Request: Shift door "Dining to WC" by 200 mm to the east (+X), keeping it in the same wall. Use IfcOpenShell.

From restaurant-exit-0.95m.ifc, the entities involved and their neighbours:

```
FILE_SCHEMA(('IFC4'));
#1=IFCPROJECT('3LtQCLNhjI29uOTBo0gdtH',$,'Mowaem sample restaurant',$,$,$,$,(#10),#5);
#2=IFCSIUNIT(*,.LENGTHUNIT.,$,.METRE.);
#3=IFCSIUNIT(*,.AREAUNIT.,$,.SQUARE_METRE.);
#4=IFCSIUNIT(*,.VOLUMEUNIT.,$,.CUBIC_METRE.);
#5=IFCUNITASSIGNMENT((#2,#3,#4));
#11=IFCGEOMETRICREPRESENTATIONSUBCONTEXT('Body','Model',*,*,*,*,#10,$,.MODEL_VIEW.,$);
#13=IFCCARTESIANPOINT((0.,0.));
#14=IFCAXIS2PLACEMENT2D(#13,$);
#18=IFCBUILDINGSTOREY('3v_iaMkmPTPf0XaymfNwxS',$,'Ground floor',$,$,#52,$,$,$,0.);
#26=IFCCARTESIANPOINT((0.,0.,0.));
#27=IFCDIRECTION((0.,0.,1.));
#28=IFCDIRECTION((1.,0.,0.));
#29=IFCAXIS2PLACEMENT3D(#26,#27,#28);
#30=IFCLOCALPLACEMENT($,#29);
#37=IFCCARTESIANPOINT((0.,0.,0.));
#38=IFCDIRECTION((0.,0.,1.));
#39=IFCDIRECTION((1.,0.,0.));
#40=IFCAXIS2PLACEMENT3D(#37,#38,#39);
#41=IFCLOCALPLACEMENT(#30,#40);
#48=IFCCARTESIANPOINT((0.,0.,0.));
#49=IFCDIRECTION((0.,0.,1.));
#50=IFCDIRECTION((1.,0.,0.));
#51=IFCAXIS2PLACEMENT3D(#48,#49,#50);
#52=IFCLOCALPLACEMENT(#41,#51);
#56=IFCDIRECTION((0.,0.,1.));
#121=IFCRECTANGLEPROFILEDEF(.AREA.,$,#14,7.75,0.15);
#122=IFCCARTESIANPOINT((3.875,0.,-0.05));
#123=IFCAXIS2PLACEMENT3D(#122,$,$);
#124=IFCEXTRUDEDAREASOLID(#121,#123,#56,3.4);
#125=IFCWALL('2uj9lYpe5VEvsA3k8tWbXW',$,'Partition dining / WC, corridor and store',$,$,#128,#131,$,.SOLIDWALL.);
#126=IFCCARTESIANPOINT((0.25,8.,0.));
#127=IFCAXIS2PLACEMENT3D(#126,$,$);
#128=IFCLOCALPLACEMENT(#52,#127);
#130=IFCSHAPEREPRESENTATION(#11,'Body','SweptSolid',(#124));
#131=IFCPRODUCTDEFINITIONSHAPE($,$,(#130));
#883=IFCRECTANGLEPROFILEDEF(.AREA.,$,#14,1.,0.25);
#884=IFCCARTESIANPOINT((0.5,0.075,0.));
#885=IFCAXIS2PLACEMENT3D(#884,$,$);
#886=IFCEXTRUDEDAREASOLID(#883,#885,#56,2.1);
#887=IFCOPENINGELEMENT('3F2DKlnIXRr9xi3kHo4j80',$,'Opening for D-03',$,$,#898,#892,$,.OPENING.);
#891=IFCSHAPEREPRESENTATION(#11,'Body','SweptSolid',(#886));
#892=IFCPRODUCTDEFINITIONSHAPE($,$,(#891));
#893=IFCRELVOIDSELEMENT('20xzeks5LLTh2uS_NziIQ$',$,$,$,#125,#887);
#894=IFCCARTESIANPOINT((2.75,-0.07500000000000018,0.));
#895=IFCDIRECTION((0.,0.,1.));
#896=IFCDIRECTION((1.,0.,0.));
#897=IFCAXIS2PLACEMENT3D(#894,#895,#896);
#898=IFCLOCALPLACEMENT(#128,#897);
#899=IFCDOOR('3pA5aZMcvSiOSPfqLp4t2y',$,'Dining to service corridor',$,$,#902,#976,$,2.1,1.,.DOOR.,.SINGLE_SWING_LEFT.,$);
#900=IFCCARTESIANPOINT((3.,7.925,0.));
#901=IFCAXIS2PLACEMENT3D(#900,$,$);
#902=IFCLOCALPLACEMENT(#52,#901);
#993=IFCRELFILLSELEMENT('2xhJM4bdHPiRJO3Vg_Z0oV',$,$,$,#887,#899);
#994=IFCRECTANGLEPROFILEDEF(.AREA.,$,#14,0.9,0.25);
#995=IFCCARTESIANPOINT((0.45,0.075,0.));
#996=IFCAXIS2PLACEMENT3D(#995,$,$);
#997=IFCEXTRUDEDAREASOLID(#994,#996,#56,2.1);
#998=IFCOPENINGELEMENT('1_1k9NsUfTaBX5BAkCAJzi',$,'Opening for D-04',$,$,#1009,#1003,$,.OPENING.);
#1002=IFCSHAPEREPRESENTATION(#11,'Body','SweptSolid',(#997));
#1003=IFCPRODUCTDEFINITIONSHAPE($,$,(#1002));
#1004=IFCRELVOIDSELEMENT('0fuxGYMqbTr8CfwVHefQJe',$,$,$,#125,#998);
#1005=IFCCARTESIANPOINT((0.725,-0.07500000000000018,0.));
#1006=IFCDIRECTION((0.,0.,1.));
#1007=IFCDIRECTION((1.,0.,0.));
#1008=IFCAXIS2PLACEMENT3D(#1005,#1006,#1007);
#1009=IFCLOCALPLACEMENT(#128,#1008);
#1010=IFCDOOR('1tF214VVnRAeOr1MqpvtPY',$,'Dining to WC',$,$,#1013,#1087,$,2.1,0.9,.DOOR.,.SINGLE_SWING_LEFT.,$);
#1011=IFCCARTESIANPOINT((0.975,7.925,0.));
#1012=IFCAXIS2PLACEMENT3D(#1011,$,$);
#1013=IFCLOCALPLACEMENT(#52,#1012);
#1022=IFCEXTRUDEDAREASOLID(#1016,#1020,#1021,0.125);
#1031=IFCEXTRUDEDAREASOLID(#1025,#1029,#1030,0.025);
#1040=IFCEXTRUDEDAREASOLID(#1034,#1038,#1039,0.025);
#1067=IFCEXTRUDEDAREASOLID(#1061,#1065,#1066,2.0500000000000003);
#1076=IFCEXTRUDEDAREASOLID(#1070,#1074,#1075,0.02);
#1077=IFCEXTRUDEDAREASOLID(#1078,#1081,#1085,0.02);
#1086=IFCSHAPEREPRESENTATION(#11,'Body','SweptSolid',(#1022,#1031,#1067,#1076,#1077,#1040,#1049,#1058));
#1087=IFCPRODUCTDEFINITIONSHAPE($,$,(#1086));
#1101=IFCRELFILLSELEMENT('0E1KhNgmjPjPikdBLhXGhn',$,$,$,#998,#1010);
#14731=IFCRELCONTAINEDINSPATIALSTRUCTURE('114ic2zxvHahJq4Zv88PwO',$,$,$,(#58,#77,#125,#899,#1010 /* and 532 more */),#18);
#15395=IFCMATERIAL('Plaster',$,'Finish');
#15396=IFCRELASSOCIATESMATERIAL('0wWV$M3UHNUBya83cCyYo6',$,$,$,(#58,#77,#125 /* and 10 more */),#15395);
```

```python
import ifcopenshell
import ifcopenshell.api.geometry
import ifcopenshell.util.placement

model = ifcopenshell.open("restaurant-exit-0.95m.ifc")

door = model.by_id(1010)
opening = door.FillsVoids[0].RelatingOpeningElement
wall = opening.VoidsElements[0].RelatingBuildingElement

wall_matrix = ifcopenshell.util.placement.get_local_placement(wall.ObjectPlacement)
shift = wall_matrix[:3, 0] * 0.2
before = ifcopenshell.util.placement.get_local_placement(door.ObjectPlacement)[:3, 3].copy()

# The door is not placed relative to its opening, so move both.
for product in (opening, door):
    matrix = ifcopenshell.util.placement.get_local_placement(product.ObjectPlacement)
    matrix[:3, 3] += shift
    ifcopenshell.api.geometry.edit_object_placement(model, product=product, matrix=matrix, is_si=False)

after = ifcopenshell.util.placement.get_local_placement(door.ObjectPlacement)[:3, 3]
print("door moved by", (after - before).round(3) + 0.0)

model.write("restaurant-exit-0.95m_v2.ifc")
```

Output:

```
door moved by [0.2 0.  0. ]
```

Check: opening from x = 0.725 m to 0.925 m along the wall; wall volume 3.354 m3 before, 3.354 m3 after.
